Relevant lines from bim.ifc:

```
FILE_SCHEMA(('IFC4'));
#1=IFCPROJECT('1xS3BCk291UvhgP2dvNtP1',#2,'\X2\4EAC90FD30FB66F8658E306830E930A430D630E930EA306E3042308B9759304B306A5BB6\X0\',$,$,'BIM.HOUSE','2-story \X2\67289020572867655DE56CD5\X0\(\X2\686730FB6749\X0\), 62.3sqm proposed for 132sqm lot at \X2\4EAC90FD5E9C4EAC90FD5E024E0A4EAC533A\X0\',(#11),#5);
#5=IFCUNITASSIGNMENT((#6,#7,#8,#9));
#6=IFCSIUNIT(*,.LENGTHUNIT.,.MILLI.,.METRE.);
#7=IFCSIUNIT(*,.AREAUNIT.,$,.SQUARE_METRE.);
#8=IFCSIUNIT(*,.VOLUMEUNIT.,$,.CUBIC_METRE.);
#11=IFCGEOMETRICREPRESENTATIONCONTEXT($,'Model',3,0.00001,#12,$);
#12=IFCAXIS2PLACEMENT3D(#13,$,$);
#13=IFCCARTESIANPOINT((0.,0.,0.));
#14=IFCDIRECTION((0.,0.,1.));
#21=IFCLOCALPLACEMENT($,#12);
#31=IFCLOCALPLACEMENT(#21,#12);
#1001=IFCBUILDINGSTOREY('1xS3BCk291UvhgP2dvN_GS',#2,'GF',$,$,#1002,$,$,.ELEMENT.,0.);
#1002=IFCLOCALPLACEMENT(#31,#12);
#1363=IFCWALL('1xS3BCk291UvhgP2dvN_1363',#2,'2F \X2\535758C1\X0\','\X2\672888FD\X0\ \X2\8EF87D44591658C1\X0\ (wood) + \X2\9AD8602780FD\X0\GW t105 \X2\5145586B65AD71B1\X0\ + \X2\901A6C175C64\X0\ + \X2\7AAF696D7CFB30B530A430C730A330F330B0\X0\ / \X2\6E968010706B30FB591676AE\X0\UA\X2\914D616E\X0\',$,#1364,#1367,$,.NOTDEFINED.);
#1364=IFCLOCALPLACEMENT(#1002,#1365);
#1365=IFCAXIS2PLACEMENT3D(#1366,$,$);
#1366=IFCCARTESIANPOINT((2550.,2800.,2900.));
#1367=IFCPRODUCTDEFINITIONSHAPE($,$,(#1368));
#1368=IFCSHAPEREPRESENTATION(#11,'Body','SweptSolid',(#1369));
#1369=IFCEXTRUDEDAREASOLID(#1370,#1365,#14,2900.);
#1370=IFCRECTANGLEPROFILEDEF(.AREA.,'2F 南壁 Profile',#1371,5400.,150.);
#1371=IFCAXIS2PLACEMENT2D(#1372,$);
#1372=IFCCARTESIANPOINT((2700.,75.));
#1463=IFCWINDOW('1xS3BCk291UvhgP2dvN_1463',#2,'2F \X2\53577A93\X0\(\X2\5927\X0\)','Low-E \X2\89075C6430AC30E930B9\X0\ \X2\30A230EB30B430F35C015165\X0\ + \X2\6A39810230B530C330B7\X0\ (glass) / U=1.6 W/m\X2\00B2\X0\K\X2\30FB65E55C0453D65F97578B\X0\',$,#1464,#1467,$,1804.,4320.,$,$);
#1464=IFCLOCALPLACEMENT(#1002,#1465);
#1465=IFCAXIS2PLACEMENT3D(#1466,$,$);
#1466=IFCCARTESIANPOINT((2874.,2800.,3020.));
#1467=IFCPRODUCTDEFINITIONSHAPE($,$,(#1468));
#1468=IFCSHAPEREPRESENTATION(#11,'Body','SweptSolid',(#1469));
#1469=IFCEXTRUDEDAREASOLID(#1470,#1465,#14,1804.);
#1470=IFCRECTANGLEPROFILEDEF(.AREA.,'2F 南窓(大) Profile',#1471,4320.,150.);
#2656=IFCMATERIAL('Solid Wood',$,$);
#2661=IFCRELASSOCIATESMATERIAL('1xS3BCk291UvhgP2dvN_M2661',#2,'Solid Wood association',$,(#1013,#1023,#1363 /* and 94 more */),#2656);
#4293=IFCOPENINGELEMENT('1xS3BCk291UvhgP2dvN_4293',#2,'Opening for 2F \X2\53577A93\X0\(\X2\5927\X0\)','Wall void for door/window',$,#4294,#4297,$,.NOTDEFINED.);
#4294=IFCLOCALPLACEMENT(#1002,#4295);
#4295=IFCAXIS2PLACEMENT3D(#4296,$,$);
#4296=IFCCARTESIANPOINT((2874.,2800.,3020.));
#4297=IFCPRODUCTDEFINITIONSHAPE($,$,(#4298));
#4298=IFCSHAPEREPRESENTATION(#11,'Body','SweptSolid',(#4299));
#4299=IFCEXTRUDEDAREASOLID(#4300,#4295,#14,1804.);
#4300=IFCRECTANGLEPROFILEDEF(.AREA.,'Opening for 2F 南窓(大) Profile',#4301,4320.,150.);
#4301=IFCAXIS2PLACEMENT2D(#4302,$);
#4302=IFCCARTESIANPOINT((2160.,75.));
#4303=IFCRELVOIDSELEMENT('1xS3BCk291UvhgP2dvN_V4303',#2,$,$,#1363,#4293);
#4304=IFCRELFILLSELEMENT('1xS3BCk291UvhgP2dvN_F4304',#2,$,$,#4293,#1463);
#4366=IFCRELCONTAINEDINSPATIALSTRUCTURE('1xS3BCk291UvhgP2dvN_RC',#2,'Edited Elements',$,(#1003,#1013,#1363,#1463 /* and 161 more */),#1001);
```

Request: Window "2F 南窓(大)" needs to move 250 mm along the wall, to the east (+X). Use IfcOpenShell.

```python
import ifcopenshell
import ifcopenshell.api.geometry
import ifcopenshell.util.placement
import ifcopenshell.util.unit

model = ifcopenshell.open("bim.ifc")
unit_scale = ifcopenshell.util.unit.calculate_unit_scale(model)

window = model.by_guid("1xS3BCk291UvhgP2dvN_1463")
opening = window.FillsVoids[0].RelatingOpeningElement
wall = opening.VoidsElements[0].RelatingBuildingElement

wall_matrix = ifcopenshell.util.placement.get_local_placement(wall.ObjectPlacement)
shift = wall_matrix[:3, 0] * 0.25 / unit_scale
before = ifcopenshell.util.placement.get_local_placement(window.ObjectPlacement)[:3, 3].copy()

# The window is not placed relative to its opening, so move both.
for product in (opening, window):
    matrix = ifcopenshell.util.placement.get_local_placement(product.ObjectPlacement)
    matrix[:3, 3] += shift
    ifcopenshell.api.geometry.edit_object_placement(model, product=product, matrix=matrix, is_si=False)

after = ifcopenshell.util.placement.get_local_placement(window.ObjectPlacement)[:3, 3]
print("window moved by", (after - before).round(3) + 0.0)

model.write("bim_rev.ifc")
```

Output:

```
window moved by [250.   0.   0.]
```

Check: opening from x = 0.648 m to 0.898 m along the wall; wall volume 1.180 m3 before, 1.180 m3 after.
